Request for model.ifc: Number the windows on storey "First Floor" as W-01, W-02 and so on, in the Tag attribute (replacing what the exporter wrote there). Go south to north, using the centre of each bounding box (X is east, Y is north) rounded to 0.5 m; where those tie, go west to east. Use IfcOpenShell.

First a look at what the model holds.

```python
import ifcopenshell
import ifcopenshell.util.element
import ifcopenshell.util.placement

model = ifcopenshell.open("model.ifc")
print(model.schema)
storey = next(s for s in model.by_type("IfcBuildingStorey") if s.Name == "First Floor")
windows = [e for e in ifcopenshell.util.element.get_decomposition(storey) if e.is_a("IfcWindow")]
for e in sorted(windows, key=lambda e: e.id()):
    origin = ifcopenshell.util.placement.get_local_placement(e.ObjectPlacement)[:3, 3]
    print(e.id(), e.Tag, e.Name, origin.round(2) + 0.0, sep=" | ")
```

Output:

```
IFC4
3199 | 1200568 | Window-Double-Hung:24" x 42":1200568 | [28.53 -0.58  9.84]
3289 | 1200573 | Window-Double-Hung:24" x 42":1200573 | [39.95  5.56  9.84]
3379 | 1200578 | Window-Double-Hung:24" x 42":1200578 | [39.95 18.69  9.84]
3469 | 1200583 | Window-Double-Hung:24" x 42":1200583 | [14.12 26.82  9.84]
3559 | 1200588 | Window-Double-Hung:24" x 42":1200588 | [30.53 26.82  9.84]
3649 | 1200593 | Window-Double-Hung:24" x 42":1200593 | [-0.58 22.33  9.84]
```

```python
import ifcopenshell
import ifcopenshell.geom
import ifcopenshell.util.element
import ifcopenshell.util.shape

model = ifcopenshell.open("model.ifc")
settings = ifcopenshell.geom.settings()
settings.set("use-world-coords", True)


def centre(element):
    shape = ifcopenshell.geom.create_shape(settings, element)
    return ifcopenshell.util.shape.get_bbox_centroid(shape.geometry)


storey = next(s for s in model.by_type("IfcBuildingStorey") if s.Name == "First Floor")
windows = [e for e in ifcopenshell.util.element.get_decomposition(storey) if e.is_a("IfcWindow")]

# Insertion points can sit at a corner or the storey origin, so sort by the geometry (in metres).
centres = {e: centre(e) for e in windows}
windows.sort(key=lambda e: (round(centres[e][1] / 0.5), centres[e][0]))

for i, e in enumerate(windows, start=1):
    number = f"W-{i:02d}"
    e.Tag = number
    print(e.id(), number)

model.write("model_updated.ifc")
```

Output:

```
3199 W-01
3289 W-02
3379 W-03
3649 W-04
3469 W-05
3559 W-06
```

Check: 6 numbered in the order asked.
